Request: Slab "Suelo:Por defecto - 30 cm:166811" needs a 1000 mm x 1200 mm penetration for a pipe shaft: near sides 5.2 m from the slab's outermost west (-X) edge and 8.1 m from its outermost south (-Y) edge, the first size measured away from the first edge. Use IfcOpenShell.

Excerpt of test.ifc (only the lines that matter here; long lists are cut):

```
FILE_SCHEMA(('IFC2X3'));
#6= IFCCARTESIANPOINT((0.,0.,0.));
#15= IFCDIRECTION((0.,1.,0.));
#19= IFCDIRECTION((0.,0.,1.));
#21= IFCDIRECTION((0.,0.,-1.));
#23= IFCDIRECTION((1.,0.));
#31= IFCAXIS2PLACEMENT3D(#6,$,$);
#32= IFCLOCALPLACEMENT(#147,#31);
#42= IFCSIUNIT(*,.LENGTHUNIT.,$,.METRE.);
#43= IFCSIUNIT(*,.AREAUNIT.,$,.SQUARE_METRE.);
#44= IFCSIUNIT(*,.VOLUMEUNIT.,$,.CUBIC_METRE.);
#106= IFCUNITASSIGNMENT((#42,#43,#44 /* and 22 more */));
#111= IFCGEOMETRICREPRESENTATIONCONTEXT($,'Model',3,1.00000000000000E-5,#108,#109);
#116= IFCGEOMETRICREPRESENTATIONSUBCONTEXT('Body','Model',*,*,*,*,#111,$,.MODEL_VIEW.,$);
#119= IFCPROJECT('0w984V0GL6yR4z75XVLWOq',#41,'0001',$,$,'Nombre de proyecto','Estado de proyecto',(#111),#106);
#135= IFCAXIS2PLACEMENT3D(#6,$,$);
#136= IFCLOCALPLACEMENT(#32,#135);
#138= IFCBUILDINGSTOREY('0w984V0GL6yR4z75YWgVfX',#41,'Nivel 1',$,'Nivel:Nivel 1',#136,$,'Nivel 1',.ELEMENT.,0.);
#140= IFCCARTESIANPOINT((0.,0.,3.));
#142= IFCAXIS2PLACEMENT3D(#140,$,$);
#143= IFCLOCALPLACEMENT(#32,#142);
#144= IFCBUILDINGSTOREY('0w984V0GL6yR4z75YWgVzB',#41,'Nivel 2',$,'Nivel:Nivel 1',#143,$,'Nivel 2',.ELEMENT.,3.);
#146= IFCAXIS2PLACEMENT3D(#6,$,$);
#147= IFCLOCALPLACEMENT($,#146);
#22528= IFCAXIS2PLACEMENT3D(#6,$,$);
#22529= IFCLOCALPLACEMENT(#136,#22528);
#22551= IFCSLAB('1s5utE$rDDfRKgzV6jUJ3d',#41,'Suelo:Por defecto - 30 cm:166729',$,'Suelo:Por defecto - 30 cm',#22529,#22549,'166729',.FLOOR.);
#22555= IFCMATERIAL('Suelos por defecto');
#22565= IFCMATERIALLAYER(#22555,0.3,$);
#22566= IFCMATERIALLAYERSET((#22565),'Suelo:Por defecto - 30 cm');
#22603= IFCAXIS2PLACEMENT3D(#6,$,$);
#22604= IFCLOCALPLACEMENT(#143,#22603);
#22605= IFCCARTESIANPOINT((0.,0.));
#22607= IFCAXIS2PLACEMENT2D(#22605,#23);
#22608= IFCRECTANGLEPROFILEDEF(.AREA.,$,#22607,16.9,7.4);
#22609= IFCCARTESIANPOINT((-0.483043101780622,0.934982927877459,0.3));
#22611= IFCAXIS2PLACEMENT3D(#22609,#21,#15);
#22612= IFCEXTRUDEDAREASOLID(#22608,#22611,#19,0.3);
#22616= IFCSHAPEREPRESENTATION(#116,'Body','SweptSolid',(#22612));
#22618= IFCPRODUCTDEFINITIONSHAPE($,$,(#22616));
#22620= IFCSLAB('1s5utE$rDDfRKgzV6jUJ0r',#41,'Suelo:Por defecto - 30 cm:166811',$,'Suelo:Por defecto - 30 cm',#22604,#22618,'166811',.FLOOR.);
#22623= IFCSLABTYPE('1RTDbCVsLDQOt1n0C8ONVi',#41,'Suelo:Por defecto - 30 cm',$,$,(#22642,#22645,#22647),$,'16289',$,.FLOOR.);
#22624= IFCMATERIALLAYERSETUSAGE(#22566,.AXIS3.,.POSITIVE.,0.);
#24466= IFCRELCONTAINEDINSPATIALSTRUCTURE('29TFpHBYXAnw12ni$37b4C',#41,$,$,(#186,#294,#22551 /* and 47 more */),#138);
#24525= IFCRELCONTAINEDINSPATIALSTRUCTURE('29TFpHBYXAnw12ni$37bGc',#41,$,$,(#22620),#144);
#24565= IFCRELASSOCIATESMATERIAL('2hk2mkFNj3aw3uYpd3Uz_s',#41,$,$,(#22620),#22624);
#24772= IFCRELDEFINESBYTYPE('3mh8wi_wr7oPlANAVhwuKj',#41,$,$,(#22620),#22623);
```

```python
import numpy as np
import ifcopenshell
import ifcopenshell.api.feature
import ifcopenshell.api.geometry
import ifcopenshell.api.root
import ifcopenshell.geom
import ifcopenshell.util.placement
import ifcopenshell.util.representation
import ifcopenshell.util.shape
import ifcopenshell.util.unit

model = ifcopenshell.open("test.ifc")
unit_scale = ifcopenshell.util.unit.calculate_unit_scale(model)
settings = ifcopenshell.geom.settings()


def volume(element):
    """Net volume in cubic metres, openings subtracted."""
    shape = ifcopenshell.geom.create_shape(settings, element)
    return ifcopenshell.util.shape.get_volume(shape.geometry)


slab = model.by_id(22620)
before = volume(slab)

# Extent in the slab's own axes, in metres. The edges named are its -X and -Y sides.
slab_shape = ifcopenshell.geom.create_shape(settings, slab)
vertices = ifcopenshell.util.shape.get_vertices(slab_shape.geometry)
x_min, y_min, bottom = vertices.min(axis=0)
top = vertices[:, 2].max()

opening = ifcopenshell.api.root.create_entity(model, ifc_class="IfcOpeningElement", name="Pipe shaft opening")
context = ifcopenshell.util.representation.get_context(model, "Model", "Body", "MODEL_VIEW")
width, depth = 1, 1.2
outline = [(0.0, 0.0), (width, 0.0), (width, depth), (0.0, depth), (0.0, 0.0)]
# Overshoot both faces by 50 mm so the cut is clean.
shape = ifcopenshell.api.geometry.add_slab_representation(
    model, context=context, depth=top - bottom + 0.1, polyline=outline
)
ifcopenshell.api.geometry.assign_representation(model, product=opening, representation=shape)

matrix = ifcopenshell.util.placement.get_local_placement(slab.ObjectPlacement)
matrix[:, 3] = matrix @ np.append(np.array([x_min + 5.2, y_min + 8.1, bottom - 0.05]) / unit_scale, 1.0)
ifcopenshell.api.geometry.edit_object_placement(model, product=opening, matrix=matrix, is_si=False)
ifcopenshell.api.feature.add_feature(model, feature=opening, element=slab)

after = volume(slab)

print(f"slab volume {before:.3f} -> {after:.3f} m3")

model.write("test_edited.ifc")
```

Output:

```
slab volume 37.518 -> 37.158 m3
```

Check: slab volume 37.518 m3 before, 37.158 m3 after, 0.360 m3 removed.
